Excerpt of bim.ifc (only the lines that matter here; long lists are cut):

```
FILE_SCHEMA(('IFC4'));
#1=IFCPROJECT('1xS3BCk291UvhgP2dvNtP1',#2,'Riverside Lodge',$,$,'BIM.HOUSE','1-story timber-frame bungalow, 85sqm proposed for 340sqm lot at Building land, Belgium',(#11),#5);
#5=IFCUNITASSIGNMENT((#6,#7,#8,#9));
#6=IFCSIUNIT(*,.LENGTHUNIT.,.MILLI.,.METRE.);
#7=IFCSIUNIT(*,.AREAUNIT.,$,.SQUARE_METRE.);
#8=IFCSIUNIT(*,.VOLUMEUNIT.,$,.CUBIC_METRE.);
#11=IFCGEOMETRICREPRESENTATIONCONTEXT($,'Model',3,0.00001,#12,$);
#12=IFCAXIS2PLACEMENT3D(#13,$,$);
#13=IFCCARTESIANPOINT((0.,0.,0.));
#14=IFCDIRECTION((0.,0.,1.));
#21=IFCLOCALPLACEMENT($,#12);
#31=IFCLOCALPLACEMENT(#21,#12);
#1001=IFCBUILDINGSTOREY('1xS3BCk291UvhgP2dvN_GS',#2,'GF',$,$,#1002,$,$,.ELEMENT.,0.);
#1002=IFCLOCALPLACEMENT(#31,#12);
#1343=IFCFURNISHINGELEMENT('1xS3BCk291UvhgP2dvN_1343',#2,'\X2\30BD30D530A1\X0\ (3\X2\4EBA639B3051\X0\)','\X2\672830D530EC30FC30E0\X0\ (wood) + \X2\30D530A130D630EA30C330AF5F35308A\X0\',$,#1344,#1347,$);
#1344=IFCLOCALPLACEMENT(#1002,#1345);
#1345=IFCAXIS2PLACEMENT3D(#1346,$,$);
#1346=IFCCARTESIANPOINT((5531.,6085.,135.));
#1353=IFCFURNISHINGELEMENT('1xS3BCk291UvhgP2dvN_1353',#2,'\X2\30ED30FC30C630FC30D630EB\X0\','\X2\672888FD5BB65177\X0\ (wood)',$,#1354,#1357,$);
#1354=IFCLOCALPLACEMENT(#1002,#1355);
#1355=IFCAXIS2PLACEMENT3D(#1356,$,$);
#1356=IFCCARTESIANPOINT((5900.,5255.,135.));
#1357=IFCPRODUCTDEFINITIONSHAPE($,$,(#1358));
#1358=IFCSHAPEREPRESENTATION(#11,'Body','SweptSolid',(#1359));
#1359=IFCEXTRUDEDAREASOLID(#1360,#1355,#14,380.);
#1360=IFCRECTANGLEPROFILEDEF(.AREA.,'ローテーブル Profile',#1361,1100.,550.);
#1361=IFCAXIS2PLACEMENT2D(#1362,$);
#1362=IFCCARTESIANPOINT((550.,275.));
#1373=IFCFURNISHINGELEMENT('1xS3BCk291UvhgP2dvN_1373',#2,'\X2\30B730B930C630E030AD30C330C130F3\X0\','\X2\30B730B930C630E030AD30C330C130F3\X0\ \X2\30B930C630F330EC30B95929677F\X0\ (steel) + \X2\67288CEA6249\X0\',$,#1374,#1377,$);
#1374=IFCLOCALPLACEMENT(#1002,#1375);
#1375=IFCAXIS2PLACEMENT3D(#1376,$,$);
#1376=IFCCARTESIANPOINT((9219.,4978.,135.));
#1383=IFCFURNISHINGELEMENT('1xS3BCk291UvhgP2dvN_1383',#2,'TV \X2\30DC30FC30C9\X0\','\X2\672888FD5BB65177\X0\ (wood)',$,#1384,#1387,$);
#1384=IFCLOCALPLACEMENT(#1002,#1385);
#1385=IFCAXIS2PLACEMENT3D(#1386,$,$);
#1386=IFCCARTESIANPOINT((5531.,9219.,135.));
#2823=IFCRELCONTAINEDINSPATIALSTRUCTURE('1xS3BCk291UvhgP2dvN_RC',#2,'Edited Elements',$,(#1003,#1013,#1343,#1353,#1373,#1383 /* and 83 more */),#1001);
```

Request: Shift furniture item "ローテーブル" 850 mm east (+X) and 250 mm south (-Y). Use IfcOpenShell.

```python
import ifcopenshell
import ifcopenshell.api.geometry
import ifcopenshell.util.placement

model = ifcopenshell.open("bim.ifc")

item = model.by_guid("1xS3BCk291UvhgP2dvN_1353")
matrix = ifcopenshell.util.placement.get_local_placement(item.ObjectPlacement)
matrix[0, 3] += 850.0
matrix[1, 3] -= 250.0
ifcopenshell.api.geometry.edit_object_placement(model, product=item, matrix=matrix, is_si=False)

print(ifcopenshell.util.placement.get_local_placement(item.ObjectPlacement).round(3) + 0.0)

model.write("bim_updated.ifc")
```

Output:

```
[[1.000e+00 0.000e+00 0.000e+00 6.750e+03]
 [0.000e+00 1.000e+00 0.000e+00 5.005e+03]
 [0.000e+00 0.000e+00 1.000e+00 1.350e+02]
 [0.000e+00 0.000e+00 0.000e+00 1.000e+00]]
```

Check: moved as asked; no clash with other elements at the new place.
